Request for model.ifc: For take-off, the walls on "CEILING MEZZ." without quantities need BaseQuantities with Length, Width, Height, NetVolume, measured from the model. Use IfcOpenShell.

First a look at what the model holds.

```python
import ifcopenshell
import ifcopenshell.util.element
import ifcopenshell.util.unit

model = ifcopenshell.open("model.ifc")
print(model.schema)
for unit_type in ("LENGTHUNIT", "AREAUNIT", "VOLUMEUNIT"):
    print(unit_type, ifcopenshell.util.unit.calculate_unit_scale(model, unit_type))
storey = next(s for s in model.by_type("IfcBuildingStorey") if s.Name == "CEILING MEZZ.")
walls = [e for e in ifcopenshell.util.element.get_decomposition(storey) if e.is_a("IfcWall")]
for e in sorted(walls, key=lambda e: e.id()):
    print(e.id(), e.is_a(), e.Name, list(ifcopenshell.util.element.get_psets(e, qtos_only=True)), sep=" | ")
```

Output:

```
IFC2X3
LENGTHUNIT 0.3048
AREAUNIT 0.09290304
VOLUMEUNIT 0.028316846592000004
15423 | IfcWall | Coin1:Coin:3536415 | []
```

```python
import ifcopenshell
import ifcopenshell.api.pset
import ifcopenshell.geom
import ifcopenshell.util.element
import ifcopenshell.util.shape
import ifcopenshell.util.unit

model = ifcopenshell.open("model.ifc")
unit_scale = ifcopenshell.util.unit.calculate_unit_scale(model)
volume_scale = ifcopenshell.util.unit.calculate_unit_scale(model, "VOLUMEUNIT")
settings = ifcopenshell.geom.settings()

storey = next(s for s in model.by_type("IfcBuildingStorey") if s.Name == "CEILING MEZZ.")
walls = [e for e in ifcopenshell.util.element.get_decomposition(storey) if e.is_a("IfcWall")]

for e in sorted(walls, key=lambda e: e.id()):
    if ifcopenshell.util.element.get_psets(e, qtos_only=True, should_inherit=False):
        continue
    # Geometry comes back in metres, in the element's own axes.
    shape = ifcopenshell.geom.create_shape(settings, e)
    values = {
        "Length": ifcopenshell.util.shape.get_x(shape.geometry) / unit_scale,
        "Width": ifcopenshell.util.shape.get_y(shape.geometry) / unit_scale,
        "Height": ifcopenshell.util.shape.get_z(shape.geometry) / unit_scale,
        "NetVolume": ifcopenshell.util.shape.get_volume(shape.geometry) / volume_scale,
    }
    qto = ifcopenshell.api.pset.add_qto(model, product=e, name="BaseQuantities")
    ifcopenshell.api.pset.edit_qto(model, qto=qto, properties=values)
    print(e.id(), {k: round(v, 3) for k, v in values.items()})

model.write("model_edited.ifc")
```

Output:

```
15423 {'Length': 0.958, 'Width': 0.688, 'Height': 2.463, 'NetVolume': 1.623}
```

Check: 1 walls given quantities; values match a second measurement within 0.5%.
